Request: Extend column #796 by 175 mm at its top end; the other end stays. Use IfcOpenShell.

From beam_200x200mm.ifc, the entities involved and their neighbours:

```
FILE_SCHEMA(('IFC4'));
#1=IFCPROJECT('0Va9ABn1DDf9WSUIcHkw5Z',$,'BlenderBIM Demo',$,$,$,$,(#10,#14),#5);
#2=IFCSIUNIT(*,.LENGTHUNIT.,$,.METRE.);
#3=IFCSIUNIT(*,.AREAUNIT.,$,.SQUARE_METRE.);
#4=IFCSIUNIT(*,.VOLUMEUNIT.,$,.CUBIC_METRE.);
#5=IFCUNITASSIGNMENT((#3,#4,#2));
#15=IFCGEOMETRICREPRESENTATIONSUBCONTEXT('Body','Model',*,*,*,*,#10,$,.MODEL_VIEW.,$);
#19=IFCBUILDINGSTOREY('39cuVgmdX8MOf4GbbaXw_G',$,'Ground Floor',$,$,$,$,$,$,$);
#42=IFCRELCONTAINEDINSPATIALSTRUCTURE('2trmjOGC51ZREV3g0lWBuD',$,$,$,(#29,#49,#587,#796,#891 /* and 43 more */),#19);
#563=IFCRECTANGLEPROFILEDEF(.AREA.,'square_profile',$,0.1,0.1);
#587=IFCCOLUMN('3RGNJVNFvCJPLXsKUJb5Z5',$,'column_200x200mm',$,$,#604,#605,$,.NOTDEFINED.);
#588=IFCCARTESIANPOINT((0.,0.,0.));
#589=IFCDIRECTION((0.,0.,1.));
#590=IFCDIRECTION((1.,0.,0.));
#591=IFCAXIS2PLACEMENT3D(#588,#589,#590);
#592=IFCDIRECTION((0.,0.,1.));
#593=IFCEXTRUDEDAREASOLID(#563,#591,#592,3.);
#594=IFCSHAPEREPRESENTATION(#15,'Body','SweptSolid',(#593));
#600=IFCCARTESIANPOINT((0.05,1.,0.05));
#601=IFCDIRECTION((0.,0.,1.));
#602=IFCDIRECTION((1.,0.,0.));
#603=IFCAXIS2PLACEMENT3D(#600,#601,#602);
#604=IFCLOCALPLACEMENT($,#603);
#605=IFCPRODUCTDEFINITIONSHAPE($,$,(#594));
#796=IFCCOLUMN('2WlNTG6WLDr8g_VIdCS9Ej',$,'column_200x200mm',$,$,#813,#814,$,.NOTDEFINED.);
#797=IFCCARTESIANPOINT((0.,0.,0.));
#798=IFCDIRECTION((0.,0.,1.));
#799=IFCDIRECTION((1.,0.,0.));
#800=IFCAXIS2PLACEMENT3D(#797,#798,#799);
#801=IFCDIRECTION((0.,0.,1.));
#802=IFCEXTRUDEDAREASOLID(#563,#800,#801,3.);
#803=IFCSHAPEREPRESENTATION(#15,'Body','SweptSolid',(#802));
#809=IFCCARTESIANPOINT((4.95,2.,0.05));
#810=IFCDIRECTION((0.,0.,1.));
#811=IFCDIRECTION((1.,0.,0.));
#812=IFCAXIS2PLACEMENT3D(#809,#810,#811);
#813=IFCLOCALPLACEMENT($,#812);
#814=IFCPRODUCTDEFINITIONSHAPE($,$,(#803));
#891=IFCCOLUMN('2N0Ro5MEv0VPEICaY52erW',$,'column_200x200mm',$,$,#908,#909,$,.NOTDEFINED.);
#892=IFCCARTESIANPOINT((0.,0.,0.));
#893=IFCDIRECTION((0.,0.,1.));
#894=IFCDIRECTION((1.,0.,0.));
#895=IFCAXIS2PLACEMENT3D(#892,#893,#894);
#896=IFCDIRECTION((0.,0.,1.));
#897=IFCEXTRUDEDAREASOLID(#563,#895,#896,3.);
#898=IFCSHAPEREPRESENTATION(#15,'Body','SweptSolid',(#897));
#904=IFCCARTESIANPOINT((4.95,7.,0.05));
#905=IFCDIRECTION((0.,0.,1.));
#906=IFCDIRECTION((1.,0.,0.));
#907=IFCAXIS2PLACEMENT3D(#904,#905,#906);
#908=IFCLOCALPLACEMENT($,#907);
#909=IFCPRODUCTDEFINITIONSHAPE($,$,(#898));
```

```python
import ifcopenshell
import ifcopenshell.util.representation
import ifcopenshell.util.unit

model = ifcopenshell.open("beam_200x200mm.ifc")
unit_scale = ifcopenshell.util.unit.calculate_unit_scale(model)

member = model.by_guid("2WlNTG6WLDr8g_VIdCS9Ej")
change = 0.175 / unit_scale

# The extrusion runs towards the end named, so only its depth changes.
body = ifcopenshell.util.representation.get_representation(member, "Model", "Body")
solid = body.Items[0]
old_length = solid.Depth
solid.Depth += change

print(f"length {old_length:g} -> {solid.Depth:g}")

model.write("beam_200x200mm_rev.ifc")
```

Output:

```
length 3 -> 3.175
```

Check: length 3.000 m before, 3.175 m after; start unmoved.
